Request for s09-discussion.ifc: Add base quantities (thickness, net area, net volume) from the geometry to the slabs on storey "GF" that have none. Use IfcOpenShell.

First a look at what the model holds.

```python
import ifcopenshell
import ifcopenshell.util.element
import ifcopenshell.util.unit

model = ifcopenshell.open("s09-discussion.ifc")
print(model.schema)
for unit_type in ("LENGTHUNIT", "AREAUNIT", "VOLUMEUNIT"):
    print(unit_type, ifcopenshell.util.unit.calculate_unit_scale(model, unit_type))
storey = next(s for s in model.by_type("IfcBuildingStorey") if s.Name == "GF")
slabs = [e for e in ifcopenshell.util.element.get_decomposition(storey) if e.is_a("IfcSlab")]
for e in sorted(slabs, key=lambda e: e.id()):
    print(e.id(), e.is_a(), e.Name, list(ifcopenshell.util.element.get_psets(e, qtos_only=True)), sep=" | ")
```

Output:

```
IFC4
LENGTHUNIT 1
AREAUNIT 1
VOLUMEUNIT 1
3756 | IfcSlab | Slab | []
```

```python
import ifcopenshell
import ifcopenshell.api.pset
import ifcopenshell.geom
import ifcopenshell.util.element
import ifcopenshell.util.shape
import ifcopenshell.util.unit

model = ifcopenshell.open("s09-discussion.ifc")
unit_scale = ifcopenshell.util.unit.calculate_unit_scale(model)
area_scale = ifcopenshell.util.unit.calculate_unit_scale(model, "AREAUNIT")
volume_scale = ifcopenshell.util.unit.calculate_unit_scale(model, "VOLUMEUNIT")
settings = ifcopenshell.geom.settings()

storey = next(s for s in model.by_type("IfcBuildingStorey") if s.Name == "GF")
slabs = [e for e in ifcopenshell.util.element.get_decomposition(storey) if e.is_a("IfcSlab")]

for e in sorted(slabs, key=lambda e: e.id()):
    if ifcopenshell.util.element.get_psets(e, qtos_only=True, should_inherit=False):
        continue
    # Geometry comes back in metres, in the element's own axes.
    shape = ifcopenshell.geom.create_shape(settings, e)
    values = {
        "Width": ifcopenshell.util.shape.get_z(shape.geometry) / unit_scale,
        "NetArea": ifcopenshell.util.shape.get_footprint_area(shape.geometry) / area_scale,
        "NetVolume": ifcopenshell.util.shape.get_volume(shape.geometry) / volume_scale,
    }
    qto = ifcopenshell.api.pset.add_qto(model, product=e, name="Qto_SlabBaseQuantities")
    ifcopenshell.api.pset.edit_qto(model, qto=qto, properties=values)
    print(e.id(), {k: round(v, 3) for k, v in values.items()})

model.write("s09-discussion_v2.ifc")
```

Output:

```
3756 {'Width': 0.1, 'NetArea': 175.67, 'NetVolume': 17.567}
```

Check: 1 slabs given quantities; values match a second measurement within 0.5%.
